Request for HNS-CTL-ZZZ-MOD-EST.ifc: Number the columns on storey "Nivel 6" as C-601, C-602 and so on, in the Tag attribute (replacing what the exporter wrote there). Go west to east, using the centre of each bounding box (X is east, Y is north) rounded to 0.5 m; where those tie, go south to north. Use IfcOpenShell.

First a look at what the model holds.

```python
import ifcopenshell
import ifcopenshell.util.element
import ifcopenshell.util.placement

model = ifcopenshell.open("HNS-CTL-ZZZ-MOD-EST.ifc")
print(model.schema)
storey = next(s for s in model.by_type("IfcBuildingStorey") if s.Name == "Nivel 6")
columns = [e for e in ifcopenshell.util.element.get_decomposition(storey) if e.is_a("IfcColumn")]
for e in sorted(columns, key=lambda e: e.id()):
    origin = ifcopenshell.util.placement.get_local_placement(e.ObjectPlacement)[:3, 3]
    print(e.id(), e.Tag, e.Name, origin.round(2) + 0.0, sep=" | ")
```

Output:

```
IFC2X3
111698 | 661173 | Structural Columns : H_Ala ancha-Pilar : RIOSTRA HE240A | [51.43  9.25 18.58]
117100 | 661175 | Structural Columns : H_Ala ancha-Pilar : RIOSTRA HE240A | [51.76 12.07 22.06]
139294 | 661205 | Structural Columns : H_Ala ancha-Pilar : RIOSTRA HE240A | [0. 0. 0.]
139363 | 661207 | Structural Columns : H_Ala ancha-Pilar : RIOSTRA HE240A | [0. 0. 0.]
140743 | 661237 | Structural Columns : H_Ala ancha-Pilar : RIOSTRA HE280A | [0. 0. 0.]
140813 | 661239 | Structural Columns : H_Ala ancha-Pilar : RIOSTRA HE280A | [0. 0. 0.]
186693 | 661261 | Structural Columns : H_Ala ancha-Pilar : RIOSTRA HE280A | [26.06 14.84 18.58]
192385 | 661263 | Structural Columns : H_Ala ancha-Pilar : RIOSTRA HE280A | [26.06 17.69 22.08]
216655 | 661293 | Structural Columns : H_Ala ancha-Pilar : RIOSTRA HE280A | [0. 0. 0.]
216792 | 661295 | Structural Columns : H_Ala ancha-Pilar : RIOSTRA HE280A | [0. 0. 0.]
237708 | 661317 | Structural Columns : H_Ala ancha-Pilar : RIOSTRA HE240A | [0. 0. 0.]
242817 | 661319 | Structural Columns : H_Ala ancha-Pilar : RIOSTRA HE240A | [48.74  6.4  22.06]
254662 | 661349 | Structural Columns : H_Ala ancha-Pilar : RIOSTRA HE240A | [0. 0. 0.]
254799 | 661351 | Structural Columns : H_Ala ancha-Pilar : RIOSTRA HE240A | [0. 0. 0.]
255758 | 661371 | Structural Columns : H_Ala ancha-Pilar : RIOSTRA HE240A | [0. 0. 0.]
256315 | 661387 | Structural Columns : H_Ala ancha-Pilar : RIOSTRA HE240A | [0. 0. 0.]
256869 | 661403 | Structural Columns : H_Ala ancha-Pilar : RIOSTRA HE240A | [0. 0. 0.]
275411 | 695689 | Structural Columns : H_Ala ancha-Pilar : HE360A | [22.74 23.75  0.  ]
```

```python
import ifcopenshell
import ifcopenshell.geom
import ifcopenshell.util.element
import ifcopenshell.util.shape

model = ifcopenshell.open("HNS-CTL-ZZZ-MOD-EST.ifc")
settings = ifcopenshell.geom.settings()
settings.set("use-world-coords", True)


def centre(element):
    shape = ifcopenshell.geom.create_shape(settings, element)
    return ifcopenshell.util.shape.get_bbox_centroid(shape.geometry)


storey = next(s for s in model.by_type("IfcBuildingStorey") if s.Name == "Nivel 6")
columns = [e for e in ifcopenshell.util.element.get_decomposition(storey) if e.is_a("IfcColumn")]

# Insertion points can sit at a corner or the storey origin, so sort by the geometry (in metres).
centres = {e: centre(e) for e in columns}
columns.sort(key=lambda e: (round(centres[e][0] / 0.5), centres[e][1]))

for i, e in enumerate(columns, start=1):
    number = f"C-6{i:02d}"
    e.Tag = number
    print(e.id(), number)

model.write("HNS-CTL-ZZZ-MOD-EST_v2.ifc")
```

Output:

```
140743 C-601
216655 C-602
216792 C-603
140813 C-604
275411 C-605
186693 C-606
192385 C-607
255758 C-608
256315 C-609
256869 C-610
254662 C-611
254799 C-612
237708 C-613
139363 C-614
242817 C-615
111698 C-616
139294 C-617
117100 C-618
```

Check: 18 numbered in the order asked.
